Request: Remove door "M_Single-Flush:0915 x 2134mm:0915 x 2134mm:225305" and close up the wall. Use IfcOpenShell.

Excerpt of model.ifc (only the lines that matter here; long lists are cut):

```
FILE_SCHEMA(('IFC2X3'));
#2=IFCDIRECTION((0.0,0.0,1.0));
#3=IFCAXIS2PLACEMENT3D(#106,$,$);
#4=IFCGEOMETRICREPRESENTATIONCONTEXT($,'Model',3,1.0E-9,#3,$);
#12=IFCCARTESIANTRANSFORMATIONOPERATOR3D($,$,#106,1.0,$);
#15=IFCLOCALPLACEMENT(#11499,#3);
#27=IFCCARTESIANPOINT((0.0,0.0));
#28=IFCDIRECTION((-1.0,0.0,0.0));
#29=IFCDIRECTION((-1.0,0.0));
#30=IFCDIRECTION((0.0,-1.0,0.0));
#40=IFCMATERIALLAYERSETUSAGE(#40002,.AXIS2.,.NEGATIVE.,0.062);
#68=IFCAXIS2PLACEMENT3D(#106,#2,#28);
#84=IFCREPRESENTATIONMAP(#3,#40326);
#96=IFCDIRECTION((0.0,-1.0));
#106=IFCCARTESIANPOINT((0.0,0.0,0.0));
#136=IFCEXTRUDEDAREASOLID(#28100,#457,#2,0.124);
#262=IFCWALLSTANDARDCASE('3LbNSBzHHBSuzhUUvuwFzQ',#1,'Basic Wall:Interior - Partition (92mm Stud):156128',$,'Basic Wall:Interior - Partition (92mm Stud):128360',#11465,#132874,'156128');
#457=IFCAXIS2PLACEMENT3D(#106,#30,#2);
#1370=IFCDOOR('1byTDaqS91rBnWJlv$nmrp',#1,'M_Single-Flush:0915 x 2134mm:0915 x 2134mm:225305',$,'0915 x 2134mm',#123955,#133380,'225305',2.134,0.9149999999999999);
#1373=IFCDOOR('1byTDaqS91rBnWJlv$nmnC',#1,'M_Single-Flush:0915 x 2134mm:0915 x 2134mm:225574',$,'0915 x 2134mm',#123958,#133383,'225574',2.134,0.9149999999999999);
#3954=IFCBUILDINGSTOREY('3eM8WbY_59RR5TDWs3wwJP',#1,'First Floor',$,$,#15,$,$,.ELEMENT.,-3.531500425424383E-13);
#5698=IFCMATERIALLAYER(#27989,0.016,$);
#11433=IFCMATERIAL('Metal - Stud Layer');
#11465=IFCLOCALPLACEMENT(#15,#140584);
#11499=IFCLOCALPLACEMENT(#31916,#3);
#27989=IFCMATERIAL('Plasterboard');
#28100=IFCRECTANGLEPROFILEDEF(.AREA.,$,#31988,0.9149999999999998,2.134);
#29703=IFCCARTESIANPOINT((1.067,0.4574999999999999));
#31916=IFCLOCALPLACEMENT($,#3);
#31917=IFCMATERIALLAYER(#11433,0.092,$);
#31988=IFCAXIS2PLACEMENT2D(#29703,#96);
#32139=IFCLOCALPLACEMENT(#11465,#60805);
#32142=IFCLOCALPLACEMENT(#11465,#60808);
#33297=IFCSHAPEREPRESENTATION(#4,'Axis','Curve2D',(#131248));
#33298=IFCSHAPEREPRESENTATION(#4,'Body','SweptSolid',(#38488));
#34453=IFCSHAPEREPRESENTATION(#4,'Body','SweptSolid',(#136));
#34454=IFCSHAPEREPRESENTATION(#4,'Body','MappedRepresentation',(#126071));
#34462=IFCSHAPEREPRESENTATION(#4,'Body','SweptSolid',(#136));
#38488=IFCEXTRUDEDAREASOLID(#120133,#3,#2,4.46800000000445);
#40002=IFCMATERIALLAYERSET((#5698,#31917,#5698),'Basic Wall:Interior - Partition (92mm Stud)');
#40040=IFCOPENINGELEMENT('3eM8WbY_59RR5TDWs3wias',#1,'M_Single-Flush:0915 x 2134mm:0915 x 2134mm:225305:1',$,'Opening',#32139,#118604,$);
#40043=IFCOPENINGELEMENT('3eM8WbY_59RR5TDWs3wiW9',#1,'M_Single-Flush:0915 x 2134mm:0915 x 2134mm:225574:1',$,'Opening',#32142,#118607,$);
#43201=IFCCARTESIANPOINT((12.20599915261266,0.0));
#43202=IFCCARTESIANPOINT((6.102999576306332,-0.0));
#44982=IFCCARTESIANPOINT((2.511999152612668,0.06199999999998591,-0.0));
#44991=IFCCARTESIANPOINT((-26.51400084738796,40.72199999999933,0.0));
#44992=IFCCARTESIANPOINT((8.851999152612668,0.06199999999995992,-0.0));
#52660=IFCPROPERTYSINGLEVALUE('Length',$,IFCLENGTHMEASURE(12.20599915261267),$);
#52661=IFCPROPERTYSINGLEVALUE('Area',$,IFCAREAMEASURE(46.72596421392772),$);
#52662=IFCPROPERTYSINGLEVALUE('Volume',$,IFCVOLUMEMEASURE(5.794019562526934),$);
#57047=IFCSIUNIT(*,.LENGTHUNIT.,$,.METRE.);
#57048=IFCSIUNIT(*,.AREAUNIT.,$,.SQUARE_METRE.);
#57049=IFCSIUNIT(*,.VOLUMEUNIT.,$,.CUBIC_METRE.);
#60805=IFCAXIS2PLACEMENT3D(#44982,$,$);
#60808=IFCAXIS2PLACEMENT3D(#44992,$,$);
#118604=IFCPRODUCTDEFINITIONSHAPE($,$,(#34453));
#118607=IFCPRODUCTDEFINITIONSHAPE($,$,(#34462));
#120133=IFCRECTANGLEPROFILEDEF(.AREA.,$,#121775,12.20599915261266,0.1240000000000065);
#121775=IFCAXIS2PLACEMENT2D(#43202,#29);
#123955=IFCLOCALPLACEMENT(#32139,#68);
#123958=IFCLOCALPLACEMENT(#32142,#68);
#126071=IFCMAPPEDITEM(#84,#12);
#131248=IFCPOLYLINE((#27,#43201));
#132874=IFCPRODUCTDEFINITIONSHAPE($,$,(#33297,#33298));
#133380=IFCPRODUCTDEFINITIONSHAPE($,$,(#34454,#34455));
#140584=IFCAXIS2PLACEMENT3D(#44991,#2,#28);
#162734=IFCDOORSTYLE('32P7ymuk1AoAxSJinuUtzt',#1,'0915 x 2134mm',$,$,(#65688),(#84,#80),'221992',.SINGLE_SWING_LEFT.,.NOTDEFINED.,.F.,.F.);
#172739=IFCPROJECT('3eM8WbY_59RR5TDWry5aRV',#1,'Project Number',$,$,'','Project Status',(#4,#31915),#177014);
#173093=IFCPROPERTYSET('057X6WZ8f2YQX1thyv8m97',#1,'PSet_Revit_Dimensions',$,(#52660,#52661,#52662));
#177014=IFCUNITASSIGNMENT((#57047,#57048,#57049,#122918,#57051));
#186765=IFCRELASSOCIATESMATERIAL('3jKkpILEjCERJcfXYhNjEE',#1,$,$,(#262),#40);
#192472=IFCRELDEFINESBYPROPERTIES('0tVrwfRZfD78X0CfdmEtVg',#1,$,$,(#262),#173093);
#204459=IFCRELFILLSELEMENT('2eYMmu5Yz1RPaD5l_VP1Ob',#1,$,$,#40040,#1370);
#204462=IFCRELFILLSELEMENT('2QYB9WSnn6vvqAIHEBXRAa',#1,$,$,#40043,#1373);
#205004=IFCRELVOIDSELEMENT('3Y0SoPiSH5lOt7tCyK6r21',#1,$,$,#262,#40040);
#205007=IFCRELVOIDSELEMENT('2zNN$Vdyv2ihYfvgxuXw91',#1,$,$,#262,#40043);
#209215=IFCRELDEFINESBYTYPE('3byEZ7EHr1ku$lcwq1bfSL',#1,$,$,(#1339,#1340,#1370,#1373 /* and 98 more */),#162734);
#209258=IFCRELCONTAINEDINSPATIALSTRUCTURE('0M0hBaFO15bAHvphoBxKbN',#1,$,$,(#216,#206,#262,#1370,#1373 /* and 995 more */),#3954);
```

```python
import ifcopenshell
import ifcopenshell.api.feature
import ifcopenshell.api.pset
import ifcopenshell.api.root
import ifcopenshell.geom
import ifcopenshell.util.element
import ifcopenshell.util.shape
import ifcopenshell.util.unit

model = ifcopenshell.open("model.ifc")
area_scale = ifcopenshell.util.unit.calculate_unit_scale(model, "AREAUNIT")
volume_scale = ifcopenshell.util.unit.calculate_unit_scale(model, "VOLUMEUNIT")
settings = ifcopenshell.geom.settings()


def volume(element):
    """Net volume in cubic metres, openings subtracted."""
    shape = ifcopenshell.geom.create_shape(settings, element)
    return ifcopenshell.util.shape.get_volume(shape.geometry)


door = model.by_guid("1byTDaqS91rBnWJlv$nmrp")
opening = door.FillsVoids[0].RelatingOpeningElement
wall = opening.VoidsElements[0].RelatingBuildingElement
before = volume(wall)

ifcopenshell.api.root.remove_product(model, product=door)
ifcopenshell.api.feature.remove_feature(model, feature=opening)

after = volume(wall)
thickness = 0.124  # wall thickness in metres

# Update the wall's stored quantities.
pset = model.by_id(ifcopenshell.util.element.get_pset(wall, "PSet_Revit_Dimensions", should_inherit=False)["id"])
ifcopenshell.api.pset.edit_pset(model, pset=pset, properties={
    "Area": model.create_entity("IfcAreaMeasure", after / thickness / area_scale),
    "Volume": model.create_entity("IfcVolumeMeasure", after / volume_scale),
})

print(f"wall volume {before:.3f} -> {after:.3f} m3")

model.write("model_edited.ifc")
```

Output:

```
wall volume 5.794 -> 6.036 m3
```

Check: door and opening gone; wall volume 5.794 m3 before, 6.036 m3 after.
